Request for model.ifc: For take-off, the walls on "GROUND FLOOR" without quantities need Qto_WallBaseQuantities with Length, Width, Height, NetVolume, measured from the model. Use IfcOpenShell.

First a look at what the model holds.

```python
import ifcopenshell
import ifcopenshell.util.element
import ifcopenshell.util.unit

model = ifcopenshell.open("model.ifc")
print(model.schema)
for unit_type in ("LENGTHUNIT", "AREAUNIT", "VOLUMEUNIT"):
    print(unit_type, ifcopenshell.util.unit.calculate_unit_scale(model, unit_type))
storey = next(s for s in model.by_type("IfcBuildingStorey") if s.Name == "GROUND FLOOR")
walls = [e for e in ifcopenshell.util.element.get_decomposition(storey) if e.is_a("IfcWall")]
for e in sorted(walls, key=lambda e: e.id()):
    print(e.id(), e.is_a(), e.Name, list(ifcopenshell.util.element.get_psets(e, qtos_only=True)), sep=" | ")
```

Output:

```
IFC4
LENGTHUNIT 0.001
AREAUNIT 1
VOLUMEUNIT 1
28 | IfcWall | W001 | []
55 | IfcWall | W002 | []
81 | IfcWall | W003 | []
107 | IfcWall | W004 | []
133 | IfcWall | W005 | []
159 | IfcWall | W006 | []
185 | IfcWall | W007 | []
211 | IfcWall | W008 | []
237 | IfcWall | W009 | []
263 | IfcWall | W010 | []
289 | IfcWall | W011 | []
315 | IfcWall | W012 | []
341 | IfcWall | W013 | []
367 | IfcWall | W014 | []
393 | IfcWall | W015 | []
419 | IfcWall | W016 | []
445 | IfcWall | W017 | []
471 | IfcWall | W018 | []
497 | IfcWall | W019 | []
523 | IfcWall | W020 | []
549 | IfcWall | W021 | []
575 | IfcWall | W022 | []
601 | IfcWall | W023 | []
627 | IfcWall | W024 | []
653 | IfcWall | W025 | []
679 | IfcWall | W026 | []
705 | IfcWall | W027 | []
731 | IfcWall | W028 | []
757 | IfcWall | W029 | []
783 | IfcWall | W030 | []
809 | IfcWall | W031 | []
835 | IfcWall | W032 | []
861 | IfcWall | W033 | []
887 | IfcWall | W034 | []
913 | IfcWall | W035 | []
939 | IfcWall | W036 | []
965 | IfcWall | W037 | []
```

```python
import ifcopenshell
import ifcopenshell.api.pset
import ifcopenshell.geom
import ifcopenshell.util.element
import ifcopenshell.util.shape
import ifcopenshell.util.unit

model = ifcopenshell.open("model.ifc")
unit_scale = ifcopenshell.util.unit.calculate_unit_scale(model)
volume_scale = ifcopenshell.util.unit.calculate_unit_scale(model, "VOLUMEUNIT")
settings = ifcopenshell.geom.settings()

storey = next(s for s in model.by_type("IfcBuildingStorey") if s.Name == "GROUND FLOOR")
walls = [e for e in ifcopenshell.util.element.get_decomposition(storey) if e.is_a("IfcWall")]

for e in sorted(walls, key=lambda e: e.id()):
    if ifcopenshell.util.element.get_psets(e, qtos_only=True, should_inherit=False):
        continue
    # Geometry comes back in metres, in the element's own axes.
    shape = ifcopenshell.geom.create_shape(settings, e)
    values = {
        "Length": ifcopenshell.util.shape.get_x(shape.geometry) / unit_scale,
        "Width": ifcopenshell.util.shape.get_y(shape.geometry) / unit_scale,
        "Height": ifcopenshell.util.shape.get_z(shape.geometry) / unit_scale,
        "NetVolume": ifcopenshell.util.shape.get_volume(shape.geometry) / volume_scale,
    }
    qto = ifcopenshell.api.pset.add_qto(model, product=e, name="Qto_WallBaseQuantities")
    ifcopenshell.api.pset.edit_qto(model, qto=qto, properties=values)
    print(e.id(), {k: round(v, 3) for k, v in values.items()})

model.write("model_v2.ifc")
```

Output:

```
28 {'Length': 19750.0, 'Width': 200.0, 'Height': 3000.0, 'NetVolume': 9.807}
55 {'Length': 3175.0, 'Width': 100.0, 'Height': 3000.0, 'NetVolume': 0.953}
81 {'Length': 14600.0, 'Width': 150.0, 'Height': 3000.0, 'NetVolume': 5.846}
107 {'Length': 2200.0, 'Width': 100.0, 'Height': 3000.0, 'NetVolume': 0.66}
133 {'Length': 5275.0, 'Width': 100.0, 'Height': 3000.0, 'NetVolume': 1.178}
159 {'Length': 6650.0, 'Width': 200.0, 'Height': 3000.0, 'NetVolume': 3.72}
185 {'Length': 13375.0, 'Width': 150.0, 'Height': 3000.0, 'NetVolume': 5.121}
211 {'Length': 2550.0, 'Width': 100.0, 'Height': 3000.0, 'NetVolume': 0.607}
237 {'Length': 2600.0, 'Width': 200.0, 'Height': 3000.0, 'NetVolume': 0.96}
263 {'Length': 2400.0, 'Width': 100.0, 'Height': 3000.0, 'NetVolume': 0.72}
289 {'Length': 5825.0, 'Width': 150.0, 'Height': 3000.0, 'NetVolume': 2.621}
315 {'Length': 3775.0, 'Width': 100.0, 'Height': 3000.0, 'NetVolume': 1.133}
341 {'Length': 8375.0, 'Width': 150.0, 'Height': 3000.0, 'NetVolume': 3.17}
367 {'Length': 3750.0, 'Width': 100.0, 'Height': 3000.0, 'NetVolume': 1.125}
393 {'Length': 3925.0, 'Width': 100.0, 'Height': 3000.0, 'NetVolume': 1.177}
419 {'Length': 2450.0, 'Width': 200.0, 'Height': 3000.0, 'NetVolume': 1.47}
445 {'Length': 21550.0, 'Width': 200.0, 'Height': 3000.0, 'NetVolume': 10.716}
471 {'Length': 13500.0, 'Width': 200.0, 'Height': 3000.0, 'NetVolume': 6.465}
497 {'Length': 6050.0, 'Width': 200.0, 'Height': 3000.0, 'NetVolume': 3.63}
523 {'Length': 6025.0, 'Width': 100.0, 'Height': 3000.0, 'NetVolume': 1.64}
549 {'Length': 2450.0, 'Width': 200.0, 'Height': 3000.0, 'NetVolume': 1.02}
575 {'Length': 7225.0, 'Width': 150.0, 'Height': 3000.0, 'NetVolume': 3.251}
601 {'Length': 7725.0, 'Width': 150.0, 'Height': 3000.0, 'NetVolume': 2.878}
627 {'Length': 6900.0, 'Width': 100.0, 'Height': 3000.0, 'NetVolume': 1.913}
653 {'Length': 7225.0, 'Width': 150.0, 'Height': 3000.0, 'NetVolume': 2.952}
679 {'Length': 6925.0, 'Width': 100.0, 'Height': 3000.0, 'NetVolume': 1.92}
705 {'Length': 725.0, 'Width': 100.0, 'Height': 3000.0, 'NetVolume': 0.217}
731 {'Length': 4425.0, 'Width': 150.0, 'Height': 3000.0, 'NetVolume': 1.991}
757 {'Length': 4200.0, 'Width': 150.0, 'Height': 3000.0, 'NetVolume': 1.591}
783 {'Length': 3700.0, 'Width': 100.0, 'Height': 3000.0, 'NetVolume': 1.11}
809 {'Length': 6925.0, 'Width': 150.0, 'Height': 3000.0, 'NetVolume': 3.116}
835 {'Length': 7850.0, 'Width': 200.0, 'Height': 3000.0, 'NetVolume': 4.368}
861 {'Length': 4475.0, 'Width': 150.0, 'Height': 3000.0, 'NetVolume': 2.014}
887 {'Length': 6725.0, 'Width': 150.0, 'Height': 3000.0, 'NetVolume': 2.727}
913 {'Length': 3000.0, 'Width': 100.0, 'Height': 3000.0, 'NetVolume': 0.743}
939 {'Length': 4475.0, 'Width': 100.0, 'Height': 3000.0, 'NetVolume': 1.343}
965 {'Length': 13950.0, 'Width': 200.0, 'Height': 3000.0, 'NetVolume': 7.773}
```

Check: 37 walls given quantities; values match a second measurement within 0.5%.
